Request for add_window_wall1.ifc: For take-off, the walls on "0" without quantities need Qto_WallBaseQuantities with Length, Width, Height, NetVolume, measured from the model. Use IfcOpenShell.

First a look at what the model holds.

```python
import ifcopenshell
import ifcopenshell.util.element
import ifcopenshell.util.unit

model = ifcopenshell.open("add_window_wall1.ifc")
print(model.schema)
for unit_type in ("LENGTHUNIT", "AREAUNIT", "VOLUMEUNIT"):
    print(unit_type, ifcopenshell.util.unit.calculate_unit_scale(model, unit_type))
storey = next(s for s in model.by_type("IfcBuildingStorey") if s.Name == "0")
walls = [e for e in ifcopenshell.util.element.get_decomposition(storey) if e.is_a("IfcWall")]
for e in sorted(walls, key=lambda e: e.id()):
    print(e.id(), e.is_a(), e.Name, list(ifcopenshell.util.element.get_psets(e, qtos_only=True)), sep=" | ")
```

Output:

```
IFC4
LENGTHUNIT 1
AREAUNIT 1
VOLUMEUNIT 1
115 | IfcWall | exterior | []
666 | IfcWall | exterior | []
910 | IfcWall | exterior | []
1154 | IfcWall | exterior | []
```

```python
import ifcopenshell
import ifcopenshell.api.pset
import ifcopenshell.geom
import ifcopenshell.util.element
import ifcopenshell.util.shape
import ifcopenshell.util.unit

model = ifcopenshell.open("add_window_wall1.ifc")
unit_scale = ifcopenshell.util.unit.calculate_unit_scale(model)
volume_scale = ifcopenshell.util.unit.calculate_unit_scale(model, "VOLUMEUNIT")
settings = ifcopenshell.geom.settings()

storey = next(s for s in model.by_type("IfcBuildingStorey") if s.Name == "0")
walls = [e for e in ifcopenshell.util.element.get_decomposition(storey) if e.is_a("IfcWall")]

for e in sorted(walls, key=lambda e: e.id()):
    if ifcopenshell.util.element.get_psets(e, qtos_only=True, should_inherit=False):
        continue
    # Geometry comes back in metres, in the element's own axes.
    shape = ifcopenshell.geom.create_shape(settings, e)
    values = {
        "Length": ifcopenshell.util.shape.get_x(shape.geometry) / unit_scale,
        "Width": ifcopenshell.util.shape.get_y(shape.geometry) / unit_scale,
        "Height": ifcopenshell.util.shape.get_z(shape.geometry) / unit_scale,
        "NetVolume": ifcopenshell.util.shape.get_volume(shape.geometry) / volume_scale,
    }
    qto = ifcopenshell.api.pset.add_qto(model, product=e, name="Qto_WallBaseQuantities")
    ifcopenshell.api.pset.edit_qto(model, qto=qto, properties=values)
    print(e.id(), {k: round(v, 3) for k, v in values.items()})

model.write("add_window_wall1_v2.ifc")
```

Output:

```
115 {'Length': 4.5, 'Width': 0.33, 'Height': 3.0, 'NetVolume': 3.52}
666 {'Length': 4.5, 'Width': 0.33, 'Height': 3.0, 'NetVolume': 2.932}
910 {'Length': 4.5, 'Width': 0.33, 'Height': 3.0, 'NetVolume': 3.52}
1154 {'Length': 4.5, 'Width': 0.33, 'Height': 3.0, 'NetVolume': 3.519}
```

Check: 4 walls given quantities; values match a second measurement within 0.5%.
